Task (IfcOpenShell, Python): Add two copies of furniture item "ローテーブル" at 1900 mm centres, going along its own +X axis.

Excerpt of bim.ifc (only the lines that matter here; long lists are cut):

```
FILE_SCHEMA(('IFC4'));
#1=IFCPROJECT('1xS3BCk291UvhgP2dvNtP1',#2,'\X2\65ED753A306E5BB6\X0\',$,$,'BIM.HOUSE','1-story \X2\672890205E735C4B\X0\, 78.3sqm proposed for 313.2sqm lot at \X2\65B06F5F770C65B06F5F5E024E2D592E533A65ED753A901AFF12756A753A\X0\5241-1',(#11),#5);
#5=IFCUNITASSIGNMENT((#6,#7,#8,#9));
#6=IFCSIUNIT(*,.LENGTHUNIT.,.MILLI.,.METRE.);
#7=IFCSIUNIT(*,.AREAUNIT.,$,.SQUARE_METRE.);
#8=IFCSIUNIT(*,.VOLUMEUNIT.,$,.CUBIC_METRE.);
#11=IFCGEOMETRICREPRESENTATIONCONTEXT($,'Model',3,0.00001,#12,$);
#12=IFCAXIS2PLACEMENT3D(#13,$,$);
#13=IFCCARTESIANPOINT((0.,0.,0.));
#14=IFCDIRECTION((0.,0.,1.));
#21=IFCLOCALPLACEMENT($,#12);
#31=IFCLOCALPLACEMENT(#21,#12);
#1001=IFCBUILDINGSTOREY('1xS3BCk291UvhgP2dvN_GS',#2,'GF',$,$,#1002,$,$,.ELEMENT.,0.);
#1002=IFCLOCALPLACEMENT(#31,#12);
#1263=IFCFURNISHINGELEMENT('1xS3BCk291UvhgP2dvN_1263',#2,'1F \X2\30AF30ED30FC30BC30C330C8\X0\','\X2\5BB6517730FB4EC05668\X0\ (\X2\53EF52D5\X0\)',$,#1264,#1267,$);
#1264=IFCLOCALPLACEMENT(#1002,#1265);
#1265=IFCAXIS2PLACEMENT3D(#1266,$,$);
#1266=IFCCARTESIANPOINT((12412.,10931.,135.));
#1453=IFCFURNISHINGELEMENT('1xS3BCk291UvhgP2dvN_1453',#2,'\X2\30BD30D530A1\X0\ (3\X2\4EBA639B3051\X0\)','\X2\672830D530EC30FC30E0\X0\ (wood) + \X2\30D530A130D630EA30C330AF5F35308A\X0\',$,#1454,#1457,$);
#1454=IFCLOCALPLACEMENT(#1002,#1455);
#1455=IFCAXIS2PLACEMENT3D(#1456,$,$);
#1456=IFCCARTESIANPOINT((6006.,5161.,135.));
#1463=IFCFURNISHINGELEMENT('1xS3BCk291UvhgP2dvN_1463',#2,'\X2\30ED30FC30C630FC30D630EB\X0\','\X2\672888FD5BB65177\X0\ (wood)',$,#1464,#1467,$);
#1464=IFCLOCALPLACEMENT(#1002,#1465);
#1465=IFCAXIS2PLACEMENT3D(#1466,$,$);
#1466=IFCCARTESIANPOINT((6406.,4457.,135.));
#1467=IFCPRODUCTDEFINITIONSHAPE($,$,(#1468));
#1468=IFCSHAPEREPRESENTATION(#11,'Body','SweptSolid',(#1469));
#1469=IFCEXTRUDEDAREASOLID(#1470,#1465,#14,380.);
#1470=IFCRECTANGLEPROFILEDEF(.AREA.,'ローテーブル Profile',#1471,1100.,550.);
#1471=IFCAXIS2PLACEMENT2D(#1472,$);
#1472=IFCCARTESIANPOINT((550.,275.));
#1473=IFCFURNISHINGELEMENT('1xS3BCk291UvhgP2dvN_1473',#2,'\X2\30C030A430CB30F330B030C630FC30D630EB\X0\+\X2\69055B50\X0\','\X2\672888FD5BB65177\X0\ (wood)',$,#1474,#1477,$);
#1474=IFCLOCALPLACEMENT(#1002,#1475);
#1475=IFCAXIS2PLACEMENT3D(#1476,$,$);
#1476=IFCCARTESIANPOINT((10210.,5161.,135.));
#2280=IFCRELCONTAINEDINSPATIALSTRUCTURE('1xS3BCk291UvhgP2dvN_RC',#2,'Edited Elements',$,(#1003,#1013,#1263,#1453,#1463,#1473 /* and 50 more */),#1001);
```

```python
import ifcopenshell
import ifcopenshell.api.geometry
import ifcopenshell.api.root
import ifcopenshell.util.element
import ifcopenshell.util.placement
import ifcopenshell.util.unit

model = ifcopenshell.open("bim.ifc")
unit_scale = ifcopenshell.util.unit.calculate_unit_scale(model)


def reuse_history(source, copy):
    """copy_class also copies each property set's owner history, people and application; keep the originals."""
    for rel in copy.IsDefinedBy:
        if rel.is_a("IfcRelDefinesByProperties") and (history := rel.RelatingPropertyDefinition.OwnerHistory):
            rel.RelatingPropertyDefinition.OwnerHistory = source.OwnerHistory
            ifcopenshell.util.element.remove_deep2(model, history)


source = model.by_guid("1xS3BCk291UvhgP2dvN_1463")
base = ifcopenshell.util.placement.get_local_placement(source.ObjectPlacement)
step = base[:3, 0] * 1.9 / unit_scale

for i in range(1, 3):
    copy = ifcopenshell.api.root.copy_class(model, product=source)
    copy.Representation = ifcopenshell.util.element.copy_deep(
        model, source.Representation, exclude=["IfcGeometricRepresentationContext", "IfcRepresentationMap"]
    )
    reuse_history(source, copy)
    matrix = base.copy()
    matrix[:3, 3] += i * step
    print("added at", matrix[:3, 3].round(3) + 0.0)
    ifcopenshell.api.geometry.edit_object_placement(model, product=copy, matrix=matrix, is_si=False)

model.write("bim_updated.ifc")
```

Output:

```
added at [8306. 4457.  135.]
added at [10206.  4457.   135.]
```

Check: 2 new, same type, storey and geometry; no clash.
